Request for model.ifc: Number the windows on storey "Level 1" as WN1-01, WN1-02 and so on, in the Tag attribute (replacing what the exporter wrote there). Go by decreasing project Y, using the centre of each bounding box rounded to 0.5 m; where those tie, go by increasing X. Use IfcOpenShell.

First a look at what the model holds.

```python
import ifcopenshell
import ifcopenshell.util.element
import ifcopenshell.util.placement

model = ifcopenshell.open("model.ifc")
print(model.schema)
storey = next(s for s in model.by_type("IfcBuildingStorey") if s.Name == "Level 1")
windows = [e for e in ifcopenshell.util.element.get_decomposition(storey) if e.is_a("IfcWindow")]
for e in sorted(windows, key=lambda e: e.id()):
    origin = ifcopenshell.util.placement.get_local_placement(e.ObjectPlacement)[:3, 3]
    print(e.id(), e.Tag, e.Name, origin.round(2) + 0.0, sep=" | ")
```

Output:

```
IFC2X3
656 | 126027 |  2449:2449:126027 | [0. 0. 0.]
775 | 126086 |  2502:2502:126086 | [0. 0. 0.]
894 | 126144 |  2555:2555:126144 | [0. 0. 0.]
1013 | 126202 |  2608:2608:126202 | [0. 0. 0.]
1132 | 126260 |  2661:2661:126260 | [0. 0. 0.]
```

```python
import ifcopenshell
import ifcopenshell.geom
import ifcopenshell.util.element
import ifcopenshell.util.shape

model = ifcopenshell.open("model.ifc")
settings = ifcopenshell.geom.settings()
settings.set("use-world-coords", True)


def centre(element):
    shape = ifcopenshell.geom.create_shape(settings, element)
    return ifcopenshell.util.shape.get_bbox_centroid(shape.geometry)


storey = next(s for s in model.by_type("IfcBuildingStorey") if s.Name == "Level 1")
windows = [e for e in ifcopenshell.util.element.get_decomposition(storey) if e.is_a("IfcWindow")]

# Insertion points can sit at a corner or the storey origin, so sort by the geometry (in metres).
centres = {e: centre(e) for e in windows}
windows.sort(key=lambda e: (-round(centres[e][1] / 0.5), centres[e][0]))

for i, e in enumerate(windows, start=1):
    number = f"WN1-{i:02d}"
    e.Tag = number
    print(e.id(), number)

model.write("model-out.ifc")
```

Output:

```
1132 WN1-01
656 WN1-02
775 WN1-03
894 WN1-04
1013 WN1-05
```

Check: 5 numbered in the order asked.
